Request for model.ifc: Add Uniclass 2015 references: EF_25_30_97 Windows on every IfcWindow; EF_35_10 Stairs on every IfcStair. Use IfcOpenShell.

First a look at what the model holds.

```python
import ifcopenshell

model = ifcopenshell.open("model.ifc")
print(model.schema)
print("classifications:", [c.Name for c in model.by_type("IfcClassification")])
for ifc_class in ("IfcDoor", "IfcRoof", "IfcStair", "IfcWall", "IfcWindow"):
    print(ifc_class, len(model.by_type(ifc_class)))
```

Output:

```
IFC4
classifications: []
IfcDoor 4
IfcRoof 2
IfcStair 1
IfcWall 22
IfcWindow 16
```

```python
import ifcopenshell
import ifcopenshell.api.classification

model = ifcopenshell.open("model.ifc")

system = ifcopenshell.api.classification.add_classification(model, classification="Uniclass 2015")

codes = {
    "IfcWindow": ("EF_25_30_97", "Windows"),
    "IfcStair": ("EF_35_10", "Stairs"),
}
for ifc_class, (code, name) in codes.items():
    products = model.by_type(ifc_class)
    ifcopenshell.api.classification.add_reference(
        model, products=products, classification=system, identification=code, name=name
    )
    print(code, len(products))

model.write("model_updated.ifc")
```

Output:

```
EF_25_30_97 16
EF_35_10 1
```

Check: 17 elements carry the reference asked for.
